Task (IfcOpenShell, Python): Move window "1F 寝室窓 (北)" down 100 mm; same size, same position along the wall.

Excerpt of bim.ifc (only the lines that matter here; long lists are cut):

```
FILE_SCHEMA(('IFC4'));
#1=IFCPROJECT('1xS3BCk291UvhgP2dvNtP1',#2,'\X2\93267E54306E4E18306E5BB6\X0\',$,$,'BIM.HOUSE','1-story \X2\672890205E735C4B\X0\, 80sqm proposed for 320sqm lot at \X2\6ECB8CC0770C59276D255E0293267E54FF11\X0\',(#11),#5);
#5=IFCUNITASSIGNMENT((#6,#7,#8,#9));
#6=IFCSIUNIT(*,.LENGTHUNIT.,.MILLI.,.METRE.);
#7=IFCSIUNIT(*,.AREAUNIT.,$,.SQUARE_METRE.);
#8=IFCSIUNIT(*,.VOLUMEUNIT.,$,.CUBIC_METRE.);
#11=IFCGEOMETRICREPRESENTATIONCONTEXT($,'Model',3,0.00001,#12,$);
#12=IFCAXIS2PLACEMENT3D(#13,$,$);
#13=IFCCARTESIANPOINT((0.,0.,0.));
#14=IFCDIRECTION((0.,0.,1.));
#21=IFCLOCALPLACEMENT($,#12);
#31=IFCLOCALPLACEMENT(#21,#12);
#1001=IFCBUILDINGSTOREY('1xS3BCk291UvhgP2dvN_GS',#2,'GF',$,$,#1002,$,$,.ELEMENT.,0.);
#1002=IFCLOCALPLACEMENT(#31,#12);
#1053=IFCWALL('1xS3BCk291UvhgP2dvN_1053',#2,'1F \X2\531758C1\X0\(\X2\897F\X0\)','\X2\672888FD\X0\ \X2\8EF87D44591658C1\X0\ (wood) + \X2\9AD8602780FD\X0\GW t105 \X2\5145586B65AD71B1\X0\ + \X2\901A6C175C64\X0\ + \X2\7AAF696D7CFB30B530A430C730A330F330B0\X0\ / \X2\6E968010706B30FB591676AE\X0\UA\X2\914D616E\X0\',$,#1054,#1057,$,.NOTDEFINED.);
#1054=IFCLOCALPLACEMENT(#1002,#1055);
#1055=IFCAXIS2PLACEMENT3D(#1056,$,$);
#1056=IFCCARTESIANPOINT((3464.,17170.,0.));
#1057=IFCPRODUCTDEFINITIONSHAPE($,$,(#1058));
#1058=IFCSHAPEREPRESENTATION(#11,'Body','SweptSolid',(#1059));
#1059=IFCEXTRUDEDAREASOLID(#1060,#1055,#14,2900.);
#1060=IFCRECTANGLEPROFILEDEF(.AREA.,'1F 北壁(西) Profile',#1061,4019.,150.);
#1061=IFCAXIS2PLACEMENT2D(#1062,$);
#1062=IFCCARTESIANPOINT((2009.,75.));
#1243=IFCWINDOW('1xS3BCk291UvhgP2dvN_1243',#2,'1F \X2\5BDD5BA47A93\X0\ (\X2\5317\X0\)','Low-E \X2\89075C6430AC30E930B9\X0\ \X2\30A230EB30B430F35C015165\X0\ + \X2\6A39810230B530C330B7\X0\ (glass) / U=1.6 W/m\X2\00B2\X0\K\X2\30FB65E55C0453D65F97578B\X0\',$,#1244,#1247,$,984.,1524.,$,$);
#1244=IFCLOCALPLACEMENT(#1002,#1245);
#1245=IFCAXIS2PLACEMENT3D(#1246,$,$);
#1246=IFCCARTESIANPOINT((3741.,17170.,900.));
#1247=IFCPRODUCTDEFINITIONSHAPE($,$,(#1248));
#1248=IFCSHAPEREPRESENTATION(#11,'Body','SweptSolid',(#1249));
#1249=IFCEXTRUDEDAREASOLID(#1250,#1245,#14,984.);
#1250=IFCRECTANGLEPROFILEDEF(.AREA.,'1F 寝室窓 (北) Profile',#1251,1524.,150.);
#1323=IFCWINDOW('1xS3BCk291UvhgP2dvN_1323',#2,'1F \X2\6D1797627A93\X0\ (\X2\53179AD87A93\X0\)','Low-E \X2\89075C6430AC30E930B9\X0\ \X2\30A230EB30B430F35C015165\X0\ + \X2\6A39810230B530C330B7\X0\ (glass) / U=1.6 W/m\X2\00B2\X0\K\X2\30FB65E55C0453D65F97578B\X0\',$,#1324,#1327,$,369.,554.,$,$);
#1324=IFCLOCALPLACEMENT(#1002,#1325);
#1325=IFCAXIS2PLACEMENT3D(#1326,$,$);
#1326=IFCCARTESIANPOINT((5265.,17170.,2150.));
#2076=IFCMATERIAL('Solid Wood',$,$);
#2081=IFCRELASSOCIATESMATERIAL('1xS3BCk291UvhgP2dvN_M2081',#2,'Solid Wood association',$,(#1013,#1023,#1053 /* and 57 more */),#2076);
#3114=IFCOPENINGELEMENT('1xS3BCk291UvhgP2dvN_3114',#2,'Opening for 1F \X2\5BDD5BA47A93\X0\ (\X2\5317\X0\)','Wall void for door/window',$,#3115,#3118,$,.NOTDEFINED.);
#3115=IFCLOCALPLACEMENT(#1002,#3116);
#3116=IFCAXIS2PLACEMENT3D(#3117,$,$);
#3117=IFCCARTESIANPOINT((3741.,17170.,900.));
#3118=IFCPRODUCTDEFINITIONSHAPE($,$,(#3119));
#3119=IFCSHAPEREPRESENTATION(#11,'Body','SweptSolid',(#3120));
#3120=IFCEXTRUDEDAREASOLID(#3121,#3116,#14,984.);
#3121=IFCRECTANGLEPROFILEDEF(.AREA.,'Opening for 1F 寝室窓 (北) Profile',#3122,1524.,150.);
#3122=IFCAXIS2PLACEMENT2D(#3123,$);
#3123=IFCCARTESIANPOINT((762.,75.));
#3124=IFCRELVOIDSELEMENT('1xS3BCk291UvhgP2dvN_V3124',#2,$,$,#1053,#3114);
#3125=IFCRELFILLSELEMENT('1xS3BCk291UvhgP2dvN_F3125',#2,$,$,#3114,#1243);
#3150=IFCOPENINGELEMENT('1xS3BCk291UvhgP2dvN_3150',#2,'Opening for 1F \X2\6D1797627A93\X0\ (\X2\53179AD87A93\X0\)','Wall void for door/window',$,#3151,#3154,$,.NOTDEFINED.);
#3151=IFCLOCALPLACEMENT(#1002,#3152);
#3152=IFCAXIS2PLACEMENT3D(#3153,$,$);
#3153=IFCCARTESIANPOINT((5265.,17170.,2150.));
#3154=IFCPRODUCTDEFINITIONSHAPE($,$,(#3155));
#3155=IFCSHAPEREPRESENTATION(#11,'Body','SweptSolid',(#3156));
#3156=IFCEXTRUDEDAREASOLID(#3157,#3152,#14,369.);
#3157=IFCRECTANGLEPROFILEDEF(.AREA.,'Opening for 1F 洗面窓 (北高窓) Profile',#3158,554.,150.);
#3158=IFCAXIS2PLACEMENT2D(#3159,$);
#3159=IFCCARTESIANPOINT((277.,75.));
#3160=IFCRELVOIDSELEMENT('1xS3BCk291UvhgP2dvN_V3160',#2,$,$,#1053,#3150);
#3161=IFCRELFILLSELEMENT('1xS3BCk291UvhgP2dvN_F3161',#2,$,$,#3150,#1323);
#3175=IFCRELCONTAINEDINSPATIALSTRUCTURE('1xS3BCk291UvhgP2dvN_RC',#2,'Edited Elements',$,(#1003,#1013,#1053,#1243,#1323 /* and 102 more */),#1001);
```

```python
import numpy as np
import ifcopenshell
import ifcopenshell.api.geometry
import ifcopenshell.util.placement
import ifcopenshell.util.unit

model = ifcopenshell.open("bim.ifc")
unit_scale = ifcopenshell.util.unit.calculate_unit_scale(model)

window = model.by_guid("1xS3BCk291UvhgP2dvN_1243")
opening = window.FillsVoids[0].RelatingOpeningElement
dz = -0.1 / unit_scale

shift = np.array([0.0, 0.0, dz])
# The window is not placed relative to its opening, so move both.
for product in (opening, window):
    matrix = ifcopenshell.util.placement.get_local_placement(product.ObjectPlacement)
    matrix[:3, 3] += shift
    ifcopenshell.api.geometry.edit_object_placement(model, product=product, matrix=matrix, is_si=False)

print(f"moved by {dz * unit_scale:+.3f} m")

model.write("bim_rev.ifc")
```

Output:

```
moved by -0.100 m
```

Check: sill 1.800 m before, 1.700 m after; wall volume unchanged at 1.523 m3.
